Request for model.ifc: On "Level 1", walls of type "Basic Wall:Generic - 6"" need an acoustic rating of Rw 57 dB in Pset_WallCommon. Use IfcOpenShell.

First a look at what the model holds.

```python
import ifcopenshell
import ifcopenshell.util.element

model = ifcopenshell.open("model.ifc")
print(model.schema)
storey = next(s for s in model.by_type("IfcBuildingStorey") if s.Name == "Level 1")
walls = [e for e in ifcopenshell.util.element.get_decomposition(storey) if e.is_a("IfcWall")]
seen = {}
for e in walls:
    element_type = ifcopenshell.util.element.get_type(e)
    key = (element_type.Name if element_type != e and element_type else None, ifcopenshell.util.element.get_pset(e, "Pset_WallCommon", "AcousticRating"))
    seen[key] = seen.get(key, 0) + 1
for (name, value), count in sorted(seen.items(), key=str):
    print(count, "x", name, "|", value)
```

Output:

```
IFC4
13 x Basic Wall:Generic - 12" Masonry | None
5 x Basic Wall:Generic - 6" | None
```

```python
import ifcopenshell
import ifcopenshell.api.pset
import ifcopenshell.util.element

model = ifcopenshell.open("model.ifc")

storey = next(s for s in model.by_type("IfcBuildingStorey") if s.Name == "Level 1")
walls = [e for e in ifcopenshell.util.element.get_decomposition(storey) if e.is_a("IfcWall")]

count = 0
for e in walls:
    element_type = ifcopenshell.util.element.get_type(e)
    if element_type in (None, e) or element_type.Name != 'Basic Wall:Generic - 6"':
        continue
    # add_pset returns the element's existing set when there is one.
    pset = ifcopenshell.api.pset.add_pset(model, product=e, name="Pset_WallCommon")
    ifcopenshell.api.pset.edit_pset(model, pset=pset, properties={"AcousticRating": "Rw 57 dB"})
    count += 1

print(count, "walls updated")

model.write("model_updated.ifc")
```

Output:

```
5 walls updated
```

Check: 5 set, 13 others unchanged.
